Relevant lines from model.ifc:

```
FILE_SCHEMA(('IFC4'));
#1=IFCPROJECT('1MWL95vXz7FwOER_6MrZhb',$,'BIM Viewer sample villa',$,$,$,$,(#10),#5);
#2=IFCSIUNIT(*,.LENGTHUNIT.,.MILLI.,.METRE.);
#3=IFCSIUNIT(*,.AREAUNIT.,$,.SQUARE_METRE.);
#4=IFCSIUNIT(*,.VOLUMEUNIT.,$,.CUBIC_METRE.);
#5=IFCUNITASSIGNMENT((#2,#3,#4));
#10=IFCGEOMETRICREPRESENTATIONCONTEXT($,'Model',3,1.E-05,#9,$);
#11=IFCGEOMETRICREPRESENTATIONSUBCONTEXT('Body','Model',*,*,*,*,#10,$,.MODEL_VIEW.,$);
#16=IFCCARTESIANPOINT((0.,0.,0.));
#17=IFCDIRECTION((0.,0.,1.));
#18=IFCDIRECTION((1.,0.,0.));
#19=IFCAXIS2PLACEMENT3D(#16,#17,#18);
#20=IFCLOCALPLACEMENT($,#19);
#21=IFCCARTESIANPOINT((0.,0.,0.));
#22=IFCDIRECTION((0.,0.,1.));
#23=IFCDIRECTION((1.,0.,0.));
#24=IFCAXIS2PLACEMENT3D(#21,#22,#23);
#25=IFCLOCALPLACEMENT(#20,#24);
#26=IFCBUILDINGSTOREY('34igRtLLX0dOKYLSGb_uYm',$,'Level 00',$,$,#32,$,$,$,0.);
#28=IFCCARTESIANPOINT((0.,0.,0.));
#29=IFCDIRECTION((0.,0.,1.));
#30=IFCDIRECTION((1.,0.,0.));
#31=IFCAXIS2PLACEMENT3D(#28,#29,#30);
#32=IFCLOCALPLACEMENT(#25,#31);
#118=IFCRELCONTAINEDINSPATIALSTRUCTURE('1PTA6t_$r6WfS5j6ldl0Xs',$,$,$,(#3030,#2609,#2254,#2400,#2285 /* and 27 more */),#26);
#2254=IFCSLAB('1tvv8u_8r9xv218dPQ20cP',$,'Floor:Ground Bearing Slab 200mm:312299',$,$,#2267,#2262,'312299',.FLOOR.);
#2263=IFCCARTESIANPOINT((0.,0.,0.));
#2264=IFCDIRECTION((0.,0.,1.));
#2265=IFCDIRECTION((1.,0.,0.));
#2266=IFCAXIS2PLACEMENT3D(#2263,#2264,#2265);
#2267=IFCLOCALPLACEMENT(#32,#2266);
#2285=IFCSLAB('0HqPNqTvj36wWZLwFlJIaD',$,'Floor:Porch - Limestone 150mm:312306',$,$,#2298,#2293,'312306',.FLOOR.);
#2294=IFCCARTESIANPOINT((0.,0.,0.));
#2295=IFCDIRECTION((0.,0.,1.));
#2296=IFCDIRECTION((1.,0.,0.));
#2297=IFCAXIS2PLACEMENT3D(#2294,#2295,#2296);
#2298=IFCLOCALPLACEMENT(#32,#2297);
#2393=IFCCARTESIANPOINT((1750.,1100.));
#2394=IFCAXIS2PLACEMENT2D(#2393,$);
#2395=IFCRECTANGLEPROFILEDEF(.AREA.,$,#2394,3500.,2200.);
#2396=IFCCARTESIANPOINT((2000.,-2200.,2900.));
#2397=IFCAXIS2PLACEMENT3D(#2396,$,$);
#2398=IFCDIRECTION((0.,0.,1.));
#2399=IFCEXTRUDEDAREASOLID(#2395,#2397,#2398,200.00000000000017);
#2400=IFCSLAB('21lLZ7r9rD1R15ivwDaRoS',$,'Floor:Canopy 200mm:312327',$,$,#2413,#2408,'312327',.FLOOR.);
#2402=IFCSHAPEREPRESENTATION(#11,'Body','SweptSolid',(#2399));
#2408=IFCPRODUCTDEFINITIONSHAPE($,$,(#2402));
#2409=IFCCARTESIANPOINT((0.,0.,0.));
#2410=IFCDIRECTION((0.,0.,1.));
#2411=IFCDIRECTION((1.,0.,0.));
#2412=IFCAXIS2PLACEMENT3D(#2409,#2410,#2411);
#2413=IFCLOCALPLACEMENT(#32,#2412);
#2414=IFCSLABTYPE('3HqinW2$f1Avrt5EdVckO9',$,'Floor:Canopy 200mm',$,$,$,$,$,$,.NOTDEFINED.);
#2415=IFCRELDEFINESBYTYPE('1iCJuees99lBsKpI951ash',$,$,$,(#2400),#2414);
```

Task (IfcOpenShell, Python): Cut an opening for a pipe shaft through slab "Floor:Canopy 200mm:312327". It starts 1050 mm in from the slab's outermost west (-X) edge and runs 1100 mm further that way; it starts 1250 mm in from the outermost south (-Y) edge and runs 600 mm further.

```python
import numpy as np
import ifcopenshell
import ifcopenshell.api.feature
import ifcopenshell.api.geometry
import ifcopenshell.api.root
import ifcopenshell.geom
import ifcopenshell.util.placement
import ifcopenshell.util.representation
import ifcopenshell.util.shape
import ifcopenshell.util.unit

model = ifcopenshell.open("model.ifc")
unit_scale = ifcopenshell.util.unit.calculate_unit_scale(model)
settings = ifcopenshell.geom.settings()


def volume(element):
    """Net volume in cubic metres, openings subtracted."""
    shape = ifcopenshell.geom.create_shape(settings, element)
    return ifcopenshell.util.shape.get_volume(shape.geometry)


slab = model.by_guid("21lLZ7r9rD1R15ivwDaRoS")
before = volume(slab)

# Extent in the slab's own axes, in metres. The edges named are its -X and -Y sides.
slab_shape = ifcopenshell.geom.create_shape(settings, slab)
vertices = ifcopenshell.util.shape.get_vertices(slab_shape.geometry)
x_min, y_min, bottom = vertices.min(axis=0)
top = vertices[:, 2].max()

opening = ifcopenshell.api.root.create_entity(model, ifc_class="IfcOpeningElement", name="Pipe shaft opening", predefined_type="OPENING")
context = ifcopenshell.util.representation.get_context(model, "Model", "Body", "MODEL_VIEW")
width, depth = 1.1, 0.6
outline = [(0.0, 0.0), (width, 0.0), (width, depth), (0.0, depth), (0.0, 0.0)]
# Overshoot both faces by 50 mm so the cut is clean.
shape = ifcopenshell.api.geometry.add_slab_representation(
    model, context=context, depth=top - bottom + 0.1, polyline=outline
)
ifcopenshell.api.geometry.assign_representation(model, product=opening, representation=shape)

matrix = ifcopenshell.util.placement.get_local_placement(slab.ObjectPlacement)
matrix[:, 3] = matrix @ np.append(np.array([x_min + 1.05, y_min + 1.25, bottom - 0.05]) / unit_scale, 1.0)
ifcopenshell.api.geometry.edit_object_placement(model, product=opening, matrix=matrix, is_si=False)
ifcopenshell.api.feature.add_feature(model, feature=opening, element=slab)

after = volume(slab)

print(f"slab volume {before:.3f} -> {after:.3f} m3")

model.write("model_updated.ifc")
```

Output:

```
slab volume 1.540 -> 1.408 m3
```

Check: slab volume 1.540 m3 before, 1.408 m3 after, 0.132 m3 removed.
